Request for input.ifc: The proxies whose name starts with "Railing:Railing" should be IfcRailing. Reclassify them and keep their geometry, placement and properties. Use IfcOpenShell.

First a look at what the model holds.

```python
import re

import ifcopenshell

model = ifcopenshell.open("input.ifc")
print(model.schema)
seen = {}
for e in model.by_type("IfcBuildingElementProxy"):
    name = re.sub(r":\d+(:\d+)?$", "", e.Name or "")  # drop the element id that some exporters append
    seen[name] = seen.get(name, 0) + 1
for name, count in sorted(seen.items()):
    print(count, "x", name)
```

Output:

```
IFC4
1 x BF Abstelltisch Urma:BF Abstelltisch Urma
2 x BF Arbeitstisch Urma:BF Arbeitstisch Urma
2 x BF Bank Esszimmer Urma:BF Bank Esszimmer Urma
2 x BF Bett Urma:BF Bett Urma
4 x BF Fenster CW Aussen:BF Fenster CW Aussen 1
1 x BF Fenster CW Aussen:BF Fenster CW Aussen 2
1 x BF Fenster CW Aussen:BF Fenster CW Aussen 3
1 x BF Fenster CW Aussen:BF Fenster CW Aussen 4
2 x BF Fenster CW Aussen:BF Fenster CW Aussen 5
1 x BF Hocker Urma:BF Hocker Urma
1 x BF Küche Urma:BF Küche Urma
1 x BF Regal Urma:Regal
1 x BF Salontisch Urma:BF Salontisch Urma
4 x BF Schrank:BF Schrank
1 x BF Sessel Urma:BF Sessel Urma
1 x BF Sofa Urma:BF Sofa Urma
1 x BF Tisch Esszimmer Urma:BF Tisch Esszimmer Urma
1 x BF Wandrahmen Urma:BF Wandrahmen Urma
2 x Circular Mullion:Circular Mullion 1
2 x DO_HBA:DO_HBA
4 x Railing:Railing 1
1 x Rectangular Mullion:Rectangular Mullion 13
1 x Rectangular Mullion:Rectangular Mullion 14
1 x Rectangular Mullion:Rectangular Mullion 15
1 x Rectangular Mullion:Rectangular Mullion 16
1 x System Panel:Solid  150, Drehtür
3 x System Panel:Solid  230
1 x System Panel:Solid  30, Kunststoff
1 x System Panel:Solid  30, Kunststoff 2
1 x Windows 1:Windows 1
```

```python
import ifcopenshell
import ifcopenshell.api.root

model = ifcopenshell.open("input.ifc")

proxies = [e.id() for e in model.by_type("IfcBuildingElementProxy") if (e.Name or "").startswith("Railing:Railing")]
for step_id in proxies:
    proxy = model.by_id(step_id)
    ifcopenshell.api.root.reassign_class(model, product=proxy, ifc_class="IfcRailing")

print(sum(model.by_id(i).is_a("IfcRailing") for i in proxies), "reclassified")

model.write("input_edited.ifc")
```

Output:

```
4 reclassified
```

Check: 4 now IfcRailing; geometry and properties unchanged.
